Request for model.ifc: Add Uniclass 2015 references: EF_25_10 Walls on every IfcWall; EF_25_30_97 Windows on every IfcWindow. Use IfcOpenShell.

First a look at what the model holds.

```python
import ifcopenshell

model = ifcopenshell.open("model.ifc")
print(model.schema)
print("classifications:", [c.Name for c in model.by_type("IfcClassification")])
for ifc_class in ("IfcDoor", "IfcRoof", "IfcStair", "IfcWall", "IfcWindow"):
    print(ifc_class, len(model.by_type(ifc_class)))
```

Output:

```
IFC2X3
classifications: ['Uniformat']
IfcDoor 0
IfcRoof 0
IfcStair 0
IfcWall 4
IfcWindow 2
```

```python
import ifcopenshell
import ifcopenshell.api.classification

model = ifcopenshell.open("model.ifc")

# IFC2X3 requires Source and Edition and has no link from the project to the system.
system = model.create_entity("IfcClassification", Source="NBS", Edition="2015", Name="Uniclass 2015")

codes = {
    "IfcWall": ("EF_25_10", "Walls"),
    "IfcWindow": ("EF_25_30_97", "Windows"),
}
for ifc_class, (code, name) in codes.items():
    products = model.by_type(ifc_class)
    ifcopenshell.api.classification.add_reference(
        model, products=products, classification=system, identification=code, name=name
    )
    print(code, len(products))

model.write("model_v2.ifc")
```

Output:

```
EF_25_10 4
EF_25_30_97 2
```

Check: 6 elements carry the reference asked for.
